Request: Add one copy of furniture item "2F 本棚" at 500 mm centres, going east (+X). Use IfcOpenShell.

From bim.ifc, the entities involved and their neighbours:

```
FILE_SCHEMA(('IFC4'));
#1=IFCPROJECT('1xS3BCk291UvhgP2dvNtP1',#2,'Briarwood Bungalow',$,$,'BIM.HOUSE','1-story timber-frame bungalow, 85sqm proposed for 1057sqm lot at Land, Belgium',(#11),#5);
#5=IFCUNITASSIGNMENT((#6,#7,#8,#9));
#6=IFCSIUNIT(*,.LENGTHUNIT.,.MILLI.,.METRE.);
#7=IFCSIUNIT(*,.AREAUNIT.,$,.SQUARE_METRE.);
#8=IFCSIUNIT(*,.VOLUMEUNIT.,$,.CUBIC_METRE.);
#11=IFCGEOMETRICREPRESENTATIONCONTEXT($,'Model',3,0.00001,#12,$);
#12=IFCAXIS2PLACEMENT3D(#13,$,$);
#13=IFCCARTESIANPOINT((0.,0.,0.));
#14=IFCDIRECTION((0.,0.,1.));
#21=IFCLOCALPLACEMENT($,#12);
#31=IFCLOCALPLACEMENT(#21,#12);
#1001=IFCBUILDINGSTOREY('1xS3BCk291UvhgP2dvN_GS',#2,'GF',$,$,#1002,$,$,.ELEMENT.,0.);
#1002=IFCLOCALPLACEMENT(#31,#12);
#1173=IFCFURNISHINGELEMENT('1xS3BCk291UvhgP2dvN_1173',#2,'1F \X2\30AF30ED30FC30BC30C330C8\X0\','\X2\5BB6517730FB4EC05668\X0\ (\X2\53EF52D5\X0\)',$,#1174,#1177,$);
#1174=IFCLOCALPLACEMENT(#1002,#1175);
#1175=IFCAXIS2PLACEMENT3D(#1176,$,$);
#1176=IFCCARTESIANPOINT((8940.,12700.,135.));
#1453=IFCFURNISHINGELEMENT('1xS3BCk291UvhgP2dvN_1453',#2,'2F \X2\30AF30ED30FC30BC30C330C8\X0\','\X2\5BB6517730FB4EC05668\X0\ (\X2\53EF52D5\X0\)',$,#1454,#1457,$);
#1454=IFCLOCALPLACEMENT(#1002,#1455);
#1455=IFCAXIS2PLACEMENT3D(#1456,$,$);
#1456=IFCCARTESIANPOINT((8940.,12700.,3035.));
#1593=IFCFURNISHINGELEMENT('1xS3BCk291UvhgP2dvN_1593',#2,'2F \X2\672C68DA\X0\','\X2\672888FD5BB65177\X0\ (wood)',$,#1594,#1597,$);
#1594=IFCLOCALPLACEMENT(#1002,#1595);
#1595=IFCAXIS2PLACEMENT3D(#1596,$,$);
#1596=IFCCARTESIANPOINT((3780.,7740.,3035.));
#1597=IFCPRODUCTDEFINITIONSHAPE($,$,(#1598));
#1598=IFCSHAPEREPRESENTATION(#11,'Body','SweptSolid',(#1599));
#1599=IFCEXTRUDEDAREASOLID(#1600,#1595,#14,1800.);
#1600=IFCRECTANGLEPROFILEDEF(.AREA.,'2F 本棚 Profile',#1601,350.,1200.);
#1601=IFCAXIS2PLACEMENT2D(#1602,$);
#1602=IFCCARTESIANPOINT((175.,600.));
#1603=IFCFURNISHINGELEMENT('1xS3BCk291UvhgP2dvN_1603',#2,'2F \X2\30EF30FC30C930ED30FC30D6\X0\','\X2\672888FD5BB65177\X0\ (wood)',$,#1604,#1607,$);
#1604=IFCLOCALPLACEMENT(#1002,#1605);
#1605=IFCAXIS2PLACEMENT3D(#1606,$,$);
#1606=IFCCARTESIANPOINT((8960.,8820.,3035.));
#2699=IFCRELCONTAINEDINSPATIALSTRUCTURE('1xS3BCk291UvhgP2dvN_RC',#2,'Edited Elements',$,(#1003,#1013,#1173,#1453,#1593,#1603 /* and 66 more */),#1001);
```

```python
import numpy as np
import ifcopenshell
import ifcopenshell.api.geometry
import ifcopenshell.api.root
import ifcopenshell.util.element
import ifcopenshell.util.placement
import ifcopenshell.util.unit

model = ifcopenshell.open("bim.ifc")
unit_scale = ifcopenshell.util.unit.calculate_unit_scale(model)


def reuse_history(source, copy):
    """copy_class also copies each property set's owner history, people and application; keep the originals."""
    for rel in copy.IsDefinedBy:
        if rel.is_a("IfcRelDefinesByProperties") and (history := rel.RelatingPropertyDefinition.OwnerHistory):
            rel.RelatingPropertyDefinition.OwnerHistory = source.OwnerHistory
            ifcopenshell.util.element.remove_deep2(model, history)


source = model.by_guid("1xS3BCk291UvhgP2dvN_1593")
base = ifcopenshell.util.placement.get_local_placement(source.ObjectPlacement)
step = np.array([1.0, 0.0, 0.0]) * 0.5 / unit_scale

for i in range(1, 2):
    copy = ifcopenshell.api.root.copy_class(model, product=source)
    copy.Representation = ifcopenshell.util.element.copy_deep(
        model, source.Representation, exclude=["IfcGeometricRepresentationContext", "IfcRepresentationMap"]
    )
    reuse_history(source, copy)
    matrix = base.copy()
    matrix[:3, 3] += i * step
    print("added at", matrix[:3, 3].round(3) + 0.0)
    ifcopenshell.api.geometry.edit_object_placement(model, product=copy, matrix=matrix, is_si=False)

model.write("bim-out.ifc")
```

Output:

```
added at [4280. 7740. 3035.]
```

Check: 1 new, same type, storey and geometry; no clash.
